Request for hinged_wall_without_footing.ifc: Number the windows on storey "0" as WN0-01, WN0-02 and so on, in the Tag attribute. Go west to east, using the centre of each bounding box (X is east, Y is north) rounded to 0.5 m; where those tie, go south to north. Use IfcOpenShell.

First a look at what the model holds.

```python
import ifcopenshell
import ifcopenshell.util.element
import ifcopenshell.util.placement

model = ifcopenshell.open("hinged_wall_without_footing.ifc")
print(model.schema)
storey = next(s for s in model.by_type("IfcBuildingStorey") if s.Name == "0")
windows = [e for e in ifcopenshell.util.element.get_decomposition(storey) if e.is_a("IfcWindow")]
for e in sorted(windows, key=lambda e: e.id()):
    origin = ifcopenshell.util.placement.get_local_placement(e.ObjectPlacement)[:3, 3]
    print(e.id(), e.Tag, e.Name, origin.round(2) + 0.0, sep=" | ")
```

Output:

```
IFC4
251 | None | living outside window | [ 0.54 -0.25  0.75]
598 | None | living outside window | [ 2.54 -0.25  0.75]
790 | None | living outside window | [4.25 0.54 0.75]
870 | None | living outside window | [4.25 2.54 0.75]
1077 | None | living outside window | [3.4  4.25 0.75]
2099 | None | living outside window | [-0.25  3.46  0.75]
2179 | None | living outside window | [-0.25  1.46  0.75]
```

```python
import ifcopenshell
import ifcopenshell.geom
import ifcopenshell.util.element
import ifcopenshell.util.shape

model = ifcopenshell.open("hinged_wall_without_footing.ifc")
settings = ifcopenshell.geom.settings()
settings.set("use-world-coords", True)


def centre(element):
    shape = ifcopenshell.geom.create_shape(settings, element)
    return ifcopenshell.util.shape.get_bbox_centroid(shape.geometry)


storey = next(s for s in model.by_type("IfcBuildingStorey") if s.Name == "0")
windows = [e for e in ifcopenshell.util.element.get_decomposition(storey) if e.is_a("IfcWindow")]

# Insertion points can sit at a corner or the storey origin, so sort by the geometry (in metres).
centres = {e: centre(e) for e in windows}
windows.sort(key=lambda e: (round(centres[e][0] / 0.5), centres[e][1]))

for i, e in enumerate(windows, start=1):
    number = f"WN0-{i:02d}"
    e.Tag = number
    print(e.id(), number)

model.write("hinged_wall_without_footing_updated.ifc")
```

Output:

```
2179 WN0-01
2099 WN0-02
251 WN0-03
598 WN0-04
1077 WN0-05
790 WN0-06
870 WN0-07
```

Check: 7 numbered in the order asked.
